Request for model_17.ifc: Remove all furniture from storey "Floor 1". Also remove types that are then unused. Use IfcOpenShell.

First a look at what the model holds.

```python
import ifcopenshell
import ifcopenshell.util.element

model = ifcopenshell.open("model_17.ifc")
print(model.schema)
storey = next(s for s in model.by_type("IfcBuildingStorey") if s.Name == "Floor 1")
furniture = [e for e in ifcopenshell.util.element.get_decomposition(storey) if e.is_a("IfcFurnishingElement")]
seen = {}
for e in furniture:
    element_type = ifcopenshell.util.element.get_type(e)
    name = element_type.Name if element_type not in (None, e) else None
    seen[name] = seen.get(name, 0) + 1
for name, count in sorted(seen.items(), key=str):
    print(count, "x", name)
```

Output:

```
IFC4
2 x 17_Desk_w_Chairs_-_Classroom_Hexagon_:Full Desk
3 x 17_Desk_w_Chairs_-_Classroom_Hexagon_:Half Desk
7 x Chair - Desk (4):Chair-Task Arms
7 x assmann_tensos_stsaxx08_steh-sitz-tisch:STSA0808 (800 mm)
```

```python
import ifcopenshell
import ifcopenshell.api.root
import ifcopenshell.util.element

model = ifcopenshell.open("model_17.ifc")

storey = next(s for s in model.by_type("IfcBuildingStorey") if s.Name == "Floor 1")
furniture = [e for e in ifcopenshell.util.element.get_decomposition(storey) if e.is_a("IfcFurnishingElement")]
types = {ifcopenshell.util.element.get_type(e) for e in furniture} - {None, *furniture}

for e in furniture:
    ifcopenshell.api.root.remove_product(model, product=e)
print(len(furniture), "removed")

unused = [t for t in types if not ifcopenshell.util.element.get_types(t)]
for t in unused:
    ifcopenshell.api.root.remove_product(model, product=t)
print(len(unused), "unused types removed")

model.write("model_17-out.ifc")
```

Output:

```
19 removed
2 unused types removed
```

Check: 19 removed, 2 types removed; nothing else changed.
